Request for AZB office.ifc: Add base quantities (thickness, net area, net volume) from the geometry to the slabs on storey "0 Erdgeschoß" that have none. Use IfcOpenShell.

First a look at what the model holds.

```python
import ifcopenshell
import ifcopenshell.util.element
import ifcopenshell.util.unit

model = ifcopenshell.open("AZB office.ifc")
print(model.schema)
for unit_type in ("LENGTHUNIT", "AREAUNIT", "VOLUMEUNIT"):
    print(unit_type, ifcopenshell.util.unit.calculate_unit_scale(model, unit_type))
storey = next(s for s in model.by_type("IfcBuildingStorey") if s.Name == "0 Erdgeschoß")
slabs = [e for e in ifcopenshell.util.element.get_decomposition(storey) if e.is_a("IfcSlab")]
for e in sorted(slabs, key=lambda e: e.id()):
    print(e.id(), e.is_a(), e.Name, list(ifcopenshell.util.element.get_psets(e, qtos_only=True)), sep=" | ")
```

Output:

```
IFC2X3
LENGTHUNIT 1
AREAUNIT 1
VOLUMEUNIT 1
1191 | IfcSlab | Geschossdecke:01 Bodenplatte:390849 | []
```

```python
import ifcopenshell
import ifcopenshell.api.pset
import ifcopenshell.geom
import ifcopenshell.util.element
import ifcopenshell.util.shape
import ifcopenshell.util.unit

model = ifcopenshell.open("AZB office.ifc")
unit_scale = ifcopenshell.util.unit.calculate_unit_scale(model)
area_scale = ifcopenshell.util.unit.calculate_unit_scale(model, "AREAUNIT")
volume_scale = ifcopenshell.util.unit.calculate_unit_scale(model, "VOLUMEUNIT")
settings = ifcopenshell.geom.settings()

storey = next(s for s in model.by_type("IfcBuildingStorey") if s.Name == "0 Erdgeschoß")
slabs = [e for e in ifcopenshell.util.element.get_decomposition(storey) if e.is_a("IfcSlab")]

for e in sorted(slabs, key=lambda e: e.id()):
    if ifcopenshell.util.element.get_psets(e, qtos_only=True, should_inherit=False):
        continue
    # Geometry comes back in metres, in the element's own axes.
    shape = ifcopenshell.geom.create_shape(settings, e)
    values = {
        "Width": ifcopenshell.util.shape.get_z(shape.geometry) / unit_scale,
        "NetArea": ifcopenshell.util.shape.get_footprint_area(shape.geometry) / area_scale,
        "NetVolume": ifcopenshell.util.shape.get_volume(shape.geometry) / volume_scale,
    }
    qto = ifcopenshell.api.pset.add_qto(model, product=e, name="BaseQuantities")
    ifcopenshell.api.pset.edit_qto(model, qto=qto, properties=values)
    print(e.id(), {k: round(v, 3) for k, v in values.items()})

model.write("AZB office_v2.ifc")
```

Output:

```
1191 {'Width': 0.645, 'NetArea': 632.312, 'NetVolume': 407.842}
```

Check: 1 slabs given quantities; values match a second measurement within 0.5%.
